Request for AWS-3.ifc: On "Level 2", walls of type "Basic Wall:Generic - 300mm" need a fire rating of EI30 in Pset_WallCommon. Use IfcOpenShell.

First a look at what the model holds.

```python
import ifcopenshell
import ifcopenshell.util.element

model = ifcopenshell.open("AWS-3.ifc")
print(model.schema)
storey = next(s for s in model.by_type("IfcBuildingStorey") if s.Name == "Level 2")
walls = [e for e in ifcopenshell.util.element.get_decomposition(storey) if e.is_a("IfcWall")]
seen = {}
for e in walls:
    element_type = ifcopenshell.util.element.get_type(e)
    key = (element_type.Name if element_type != e and element_type else None, ifcopenshell.util.element.get_pset(e, "Pset_WallCommon", "FireRating"))
    seen[key] = seen.get(key, 0) + 1
for (name, value), count in sorted(seen.items(), key=str):
    print(count, "x", name, "|", value)
```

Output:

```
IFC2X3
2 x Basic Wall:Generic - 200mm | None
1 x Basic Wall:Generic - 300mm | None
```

```python
import ifcopenshell
import ifcopenshell.api.pset
import ifcopenshell.util.element

model = ifcopenshell.open("AWS-3.ifc")

storey = next(s for s in model.by_type("IfcBuildingStorey") if s.Name == "Level 2")
walls = [e for e in ifcopenshell.util.element.get_decomposition(storey) if e.is_a("IfcWall")]

count = 0
for e in walls:
    element_type = ifcopenshell.util.element.get_type(e)
    if element_type in (None, e) or element_type.Name != "Basic Wall:Generic - 300mm":
        continue
    # add_pset returns the element's existing set when there is one.
    pset = ifcopenshell.api.pset.add_pset(model, product=e, name="Pset_WallCommon")
    ifcopenshell.api.pset.edit_pset(model, pset=pset, properties={"FireRating": "EI30"})
    count += 1

print(count, "walls updated")

model.write("AWS-3_edited.ifc")
```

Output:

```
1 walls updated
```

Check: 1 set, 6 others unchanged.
